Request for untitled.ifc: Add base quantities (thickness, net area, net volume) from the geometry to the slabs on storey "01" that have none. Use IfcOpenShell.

First a look at what the model holds.

```python
import ifcopenshell
import ifcopenshell.util.element
import ifcopenshell.util.unit

model = ifcopenshell.open("untitled.ifc")
print(model.schema)
for unit_type in ("LENGTHUNIT", "AREAUNIT", "VOLUMEUNIT"):
    print(unit_type, ifcopenshell.util.unit.calculate_unit_scale(model, unit_type))
storey = next(s for s in model.by_type("IfcBuildingStorey") if s.Name == "01")
slabs = [e for e in ifcopenshell.util.element.get_decomposition(storey) if e.is_a("IfcSlab")]
for e in sorted(slabs, key=lambda e: e.id()):
    print(e.id(), e.is_a(), e.Name, list(ifcopenshell.util.element.get_psets(e, qtos_only=True)), sep=" | ")
```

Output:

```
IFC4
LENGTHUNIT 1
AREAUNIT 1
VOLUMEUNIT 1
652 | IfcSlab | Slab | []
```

```python
import ifcopenshell
import ifcopenshell.api.pset
import ifcopenshell.geom
import ifcopenshell.util.element
import ifcopenshell.util.shape
import ifcopenshell.util.unit

model = ifcopenshell.open("untitled.ifc")
unit_scale = ifcopenshell.util.unit.calculate_unit_scale(model)
area_scale = ifcopenshell.util.unit.calculate_unit_scale(model, "AREAUNIT")
volume_scale = ifcopenshell.util.unit.calculate_unit_scale(model, "VOLUMEUNIT")
settings = ifcopenshell.geom.settings()

storey = next(s for s in model.by_type("IfcBuildingStorey") if s.Name == "01")
slabs = [e for e in ifcopenshell.util.element.get_decomposition(storey) if e.is_a("IfcSlab")]

for e in sorted(slabs, key=lambda e: e.id()):
    if ifcopenshell.util.element.get_psets(e, qtos_only=True, should_inherit=False):
        continue
    # Geometry comes back in metres, in the element's own axes.
    shape = ifcopenshell.geom.create_shape(settings, e)
    values = {
        "Width": ifcopenshell.util.shape.get_z(shape.geometry) / unit_scale,
        "NetArea": ifcopenshell.util.shape.get_footprint_area(shape.geometry) / area_scale,
        "NetVolume": ifcopenshell.util.shape.get_volume(shape.geometry) / volume_scale,
    }
    qto = ifcopenshell.api.pset.add_qto(model, product=e, name="Qto_SlabBaseQuantities")
    ifcopenshell.api.pset.edit_qto(model, qto=qto, properties=values)
    print(e.id(), {k: round(v, 3) for k, v in values.items()})

model.write("untitled-out.ifc")
```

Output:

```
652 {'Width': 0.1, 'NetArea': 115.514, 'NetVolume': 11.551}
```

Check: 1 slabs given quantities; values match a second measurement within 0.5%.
